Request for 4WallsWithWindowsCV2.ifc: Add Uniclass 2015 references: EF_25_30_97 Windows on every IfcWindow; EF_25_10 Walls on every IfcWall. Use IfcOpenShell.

First a look at what the model holds.

```python
import ifcopenshell

model = ifcopenshell.open("4WallsWithWindowsCV2.ifc")
print(model.schema)
print("classifications:", [c.Name for c in model.by_type("IfcClassification")])
for ifc_class in ("IfcDoor", "IfcRoof", "IfcStair", "IfcWall", "IfcWindow"):
    print(ifc_class, len(model.by_type(ifc_class)))
```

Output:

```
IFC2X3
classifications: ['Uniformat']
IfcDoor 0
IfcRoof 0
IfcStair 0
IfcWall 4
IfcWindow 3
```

```python
import ifcopenshell
import ifcopenshell.api.classification

model = ifcopenshell.open("4WallsWithWindowsCV2.ifc")

# IFC2X3 requires Source and Edition and has no link from the project to the system.
system = model.create_entity("IfcClassification", Source="NBS", Edition="2015", Name="Uniclass 2015")

codes = {
    "IfcWindow": ("EF_25_30_97", "Windows"),
    "IfcWall": ("EF_25_10", "Walls"),
}
for ifc_class, (code, name) in codes.items():
    products = model.by_type(ifc_class)
    ifcopenshell.api.classification.add_reference(
        model, products=products, classification=system, identification=code, name=name
    )
    print(code, len(products))

model.write("4WallsWithWindowsCV2_rev.ifc")
```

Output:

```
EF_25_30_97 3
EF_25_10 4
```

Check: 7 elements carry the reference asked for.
